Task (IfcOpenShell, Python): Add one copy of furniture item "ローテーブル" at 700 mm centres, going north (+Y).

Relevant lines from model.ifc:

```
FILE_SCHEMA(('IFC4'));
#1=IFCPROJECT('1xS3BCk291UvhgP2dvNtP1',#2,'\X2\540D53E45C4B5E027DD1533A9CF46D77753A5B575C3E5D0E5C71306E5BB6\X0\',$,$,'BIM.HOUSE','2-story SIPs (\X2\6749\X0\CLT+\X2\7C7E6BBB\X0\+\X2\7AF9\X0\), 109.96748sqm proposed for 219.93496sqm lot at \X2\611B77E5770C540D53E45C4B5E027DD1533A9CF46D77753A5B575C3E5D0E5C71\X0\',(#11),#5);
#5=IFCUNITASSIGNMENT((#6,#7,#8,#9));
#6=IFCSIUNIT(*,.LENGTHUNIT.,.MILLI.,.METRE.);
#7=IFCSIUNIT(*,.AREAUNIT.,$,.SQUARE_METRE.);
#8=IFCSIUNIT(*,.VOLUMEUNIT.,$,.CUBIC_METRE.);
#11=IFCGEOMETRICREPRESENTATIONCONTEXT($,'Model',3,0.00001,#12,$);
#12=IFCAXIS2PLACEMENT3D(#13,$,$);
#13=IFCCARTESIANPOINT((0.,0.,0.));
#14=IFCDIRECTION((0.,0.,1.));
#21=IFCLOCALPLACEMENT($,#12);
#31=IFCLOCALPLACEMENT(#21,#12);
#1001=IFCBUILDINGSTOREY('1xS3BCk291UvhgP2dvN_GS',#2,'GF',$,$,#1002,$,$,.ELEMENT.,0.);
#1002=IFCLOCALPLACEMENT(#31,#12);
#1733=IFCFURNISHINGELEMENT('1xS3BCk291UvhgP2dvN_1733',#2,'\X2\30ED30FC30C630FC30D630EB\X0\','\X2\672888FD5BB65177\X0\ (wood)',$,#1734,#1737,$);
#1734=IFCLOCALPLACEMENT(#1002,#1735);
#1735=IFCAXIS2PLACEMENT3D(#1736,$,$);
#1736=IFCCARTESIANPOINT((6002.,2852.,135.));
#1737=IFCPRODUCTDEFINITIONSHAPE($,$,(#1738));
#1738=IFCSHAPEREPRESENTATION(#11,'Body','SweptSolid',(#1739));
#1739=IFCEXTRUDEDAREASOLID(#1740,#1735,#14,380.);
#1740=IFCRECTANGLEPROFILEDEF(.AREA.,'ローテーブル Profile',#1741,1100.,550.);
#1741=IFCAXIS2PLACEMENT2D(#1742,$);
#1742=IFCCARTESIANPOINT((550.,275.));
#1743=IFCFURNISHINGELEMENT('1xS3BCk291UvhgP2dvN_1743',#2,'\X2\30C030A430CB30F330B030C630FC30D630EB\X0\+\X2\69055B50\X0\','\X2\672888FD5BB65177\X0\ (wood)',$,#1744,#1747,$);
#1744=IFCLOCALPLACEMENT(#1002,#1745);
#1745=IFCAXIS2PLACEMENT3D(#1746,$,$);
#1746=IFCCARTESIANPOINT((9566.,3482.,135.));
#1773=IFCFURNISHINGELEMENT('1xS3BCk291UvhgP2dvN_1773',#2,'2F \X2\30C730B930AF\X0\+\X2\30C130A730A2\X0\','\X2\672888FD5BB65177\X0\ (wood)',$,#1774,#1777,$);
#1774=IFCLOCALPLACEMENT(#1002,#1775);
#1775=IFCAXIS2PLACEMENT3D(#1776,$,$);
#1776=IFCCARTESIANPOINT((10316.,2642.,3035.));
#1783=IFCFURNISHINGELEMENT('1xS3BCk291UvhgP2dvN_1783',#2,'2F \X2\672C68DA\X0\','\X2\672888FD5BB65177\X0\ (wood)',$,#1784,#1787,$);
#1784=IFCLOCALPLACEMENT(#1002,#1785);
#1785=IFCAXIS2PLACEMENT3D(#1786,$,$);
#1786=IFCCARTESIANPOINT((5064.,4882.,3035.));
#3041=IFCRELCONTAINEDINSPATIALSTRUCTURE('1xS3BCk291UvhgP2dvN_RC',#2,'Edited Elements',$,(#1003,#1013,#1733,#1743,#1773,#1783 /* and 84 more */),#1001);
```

```python
import numpy as np
import ifcopenshell
import ifcopenshell.api.geometry
import ifcopenshell.api.root
import ifcopenshell.util.element
import ifcopenshell.util.placement

model = ifcopenshell.open("model.ifc")


def reuse_history(source, copy):
    """copy_class also copies each property set's owner history, people and application; keep the originals."""
    for rel in copy.IsDefinedBy:
        if rel.is_a("IfcRelDefinesByProperties") and (history := rel.RelatingPropertyDefinition.OwnerHistory):
            rel.RelatingPropertyDefinition.OwnerHistory = source.OwnerHistory
            ifcopenshell.util.element.remove_deep2(model, history)


source = model.by_id(1733)
base = ifcopenshell.util.placement.get_local_placement(source.ObjectPlacement)
step = np.array([0.0, 1.0, 0.0]) * 700.0

for i in range(1, 2):
    copy = ifcopenshell.api.root.copy_class(model, product=source)
    copy.Representation = ifcopenshell.util.element.copy_deep(
        model, source.Representation, exclude=["IfcGeometricRepresentationContext", "IfcRepresentationMap"]
    )
    reuse_history(source, copy)
    matrix = base.copy()
    matrix[:3, 3] += i * step
    print("added at", matrix[:3, 3].round(3) + 0.0)
    ifcopenshell.api.geometry.edit_object_placement(model, product=copy, matrix=matrix, is_si=False)

model.write("model_edited.ifc")
```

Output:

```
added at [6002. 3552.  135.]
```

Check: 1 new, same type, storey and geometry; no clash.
